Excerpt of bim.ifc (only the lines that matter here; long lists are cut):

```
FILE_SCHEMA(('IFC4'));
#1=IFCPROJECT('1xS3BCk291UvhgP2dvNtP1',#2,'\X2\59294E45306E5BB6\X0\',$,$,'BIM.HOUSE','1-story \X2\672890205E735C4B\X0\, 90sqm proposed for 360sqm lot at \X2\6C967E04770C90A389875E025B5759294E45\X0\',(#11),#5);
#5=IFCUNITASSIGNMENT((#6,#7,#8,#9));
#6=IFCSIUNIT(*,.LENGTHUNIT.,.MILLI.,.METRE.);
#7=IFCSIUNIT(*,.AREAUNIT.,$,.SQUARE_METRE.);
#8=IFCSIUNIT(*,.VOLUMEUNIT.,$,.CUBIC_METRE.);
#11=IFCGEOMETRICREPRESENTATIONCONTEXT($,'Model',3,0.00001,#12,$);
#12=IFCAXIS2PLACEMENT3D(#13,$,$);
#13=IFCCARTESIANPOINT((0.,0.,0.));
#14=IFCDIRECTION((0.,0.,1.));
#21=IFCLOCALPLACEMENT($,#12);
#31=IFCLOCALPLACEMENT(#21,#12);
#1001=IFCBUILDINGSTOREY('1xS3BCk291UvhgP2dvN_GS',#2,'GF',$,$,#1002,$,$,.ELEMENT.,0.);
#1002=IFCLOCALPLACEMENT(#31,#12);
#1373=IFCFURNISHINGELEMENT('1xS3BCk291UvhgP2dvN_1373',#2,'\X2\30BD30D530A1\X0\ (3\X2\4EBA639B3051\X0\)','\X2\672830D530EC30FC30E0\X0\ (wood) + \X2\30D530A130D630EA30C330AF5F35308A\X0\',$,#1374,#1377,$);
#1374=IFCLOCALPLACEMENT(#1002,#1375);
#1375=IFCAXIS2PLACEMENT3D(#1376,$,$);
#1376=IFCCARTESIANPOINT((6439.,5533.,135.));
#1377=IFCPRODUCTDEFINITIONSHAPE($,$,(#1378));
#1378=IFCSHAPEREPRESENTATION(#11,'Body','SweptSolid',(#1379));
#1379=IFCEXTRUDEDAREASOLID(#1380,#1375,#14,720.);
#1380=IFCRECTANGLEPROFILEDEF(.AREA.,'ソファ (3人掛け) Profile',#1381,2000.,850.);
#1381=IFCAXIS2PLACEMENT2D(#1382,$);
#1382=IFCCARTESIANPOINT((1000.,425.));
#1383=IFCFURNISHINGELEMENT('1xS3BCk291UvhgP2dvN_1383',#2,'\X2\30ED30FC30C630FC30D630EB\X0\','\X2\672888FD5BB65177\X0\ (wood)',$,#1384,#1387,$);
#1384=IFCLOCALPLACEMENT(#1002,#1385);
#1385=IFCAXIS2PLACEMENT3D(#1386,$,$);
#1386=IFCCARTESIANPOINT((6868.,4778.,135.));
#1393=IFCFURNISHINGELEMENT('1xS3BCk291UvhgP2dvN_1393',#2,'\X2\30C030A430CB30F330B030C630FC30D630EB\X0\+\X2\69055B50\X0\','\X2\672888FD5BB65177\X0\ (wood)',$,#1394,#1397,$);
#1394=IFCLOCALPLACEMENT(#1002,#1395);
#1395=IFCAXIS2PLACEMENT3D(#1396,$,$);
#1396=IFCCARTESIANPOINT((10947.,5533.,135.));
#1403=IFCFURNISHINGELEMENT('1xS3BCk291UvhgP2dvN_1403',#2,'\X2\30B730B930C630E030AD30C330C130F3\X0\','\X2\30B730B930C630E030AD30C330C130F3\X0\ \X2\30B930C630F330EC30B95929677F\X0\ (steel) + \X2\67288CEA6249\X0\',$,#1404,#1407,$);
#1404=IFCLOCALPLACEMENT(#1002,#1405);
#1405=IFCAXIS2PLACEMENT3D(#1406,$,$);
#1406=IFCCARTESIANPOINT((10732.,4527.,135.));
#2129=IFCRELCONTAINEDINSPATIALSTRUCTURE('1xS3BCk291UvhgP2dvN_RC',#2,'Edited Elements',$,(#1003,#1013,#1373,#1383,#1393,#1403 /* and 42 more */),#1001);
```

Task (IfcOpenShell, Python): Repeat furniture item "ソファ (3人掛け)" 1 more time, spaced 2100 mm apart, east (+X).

```python
import numpy as np
import ifcopenshell
import ifcopenshell.api.geometry
import ifcopenshell.api.root
import ifcopenshell.util.element
import ifcopenshell.util.placement
import ifcopenshell.util.unit

model = ifcopenshell.open("bim.ifc")
unit_scale = ifcopenshell.util.unit.calculate_unit_scale(model)


def reuse_history(source, copy):
    """copy_class also copies each property set's owner history, people and application; keep the originals."""
    for rel in copy.IsDefinedBy:
        if rel.is_a("IfcRelDefinesByProperties") and (history := rel.RelatingPropertyDefinition.OwnerHistory):
            rel.RelatingPropertyDefinition.OwnerHistory = source.OwnerHistory
            ifcopenshell.util.element.remove_deep2(model, history)


source = model.by_guid("1xS3BCk291UvhgP2dvN_1373")
base = ifcopenshell.util.placement.get_local_placement(source.ObjectPlacement)
step = np.array([1.0, 0.0, 0.0]) * 2.1 / unit_scale

for i in range(1, 2):
    copy = ifcopenshell.api.root.copy_class(model, product=source)
    copy.Representation = ifcopenshell.util.element.copy_deep(
        model, source.Representation, exclude=["IfcGeometricRepresentationContext", "IfcRepresentationMap"]
    )
    reuse_history(source, copy)
    matrix = base.copy()
    matrix[:3, 3] += i * step
    print("added at", matrix[:3, 3].round(3) + 0.0)
    ifcopenshell.api.geometry.edit_object_placement(model, product=copy, matrix=matrix, is_si=False)

model.write("bim_rev.ifc")
```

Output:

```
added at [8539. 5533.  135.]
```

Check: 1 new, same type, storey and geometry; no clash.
